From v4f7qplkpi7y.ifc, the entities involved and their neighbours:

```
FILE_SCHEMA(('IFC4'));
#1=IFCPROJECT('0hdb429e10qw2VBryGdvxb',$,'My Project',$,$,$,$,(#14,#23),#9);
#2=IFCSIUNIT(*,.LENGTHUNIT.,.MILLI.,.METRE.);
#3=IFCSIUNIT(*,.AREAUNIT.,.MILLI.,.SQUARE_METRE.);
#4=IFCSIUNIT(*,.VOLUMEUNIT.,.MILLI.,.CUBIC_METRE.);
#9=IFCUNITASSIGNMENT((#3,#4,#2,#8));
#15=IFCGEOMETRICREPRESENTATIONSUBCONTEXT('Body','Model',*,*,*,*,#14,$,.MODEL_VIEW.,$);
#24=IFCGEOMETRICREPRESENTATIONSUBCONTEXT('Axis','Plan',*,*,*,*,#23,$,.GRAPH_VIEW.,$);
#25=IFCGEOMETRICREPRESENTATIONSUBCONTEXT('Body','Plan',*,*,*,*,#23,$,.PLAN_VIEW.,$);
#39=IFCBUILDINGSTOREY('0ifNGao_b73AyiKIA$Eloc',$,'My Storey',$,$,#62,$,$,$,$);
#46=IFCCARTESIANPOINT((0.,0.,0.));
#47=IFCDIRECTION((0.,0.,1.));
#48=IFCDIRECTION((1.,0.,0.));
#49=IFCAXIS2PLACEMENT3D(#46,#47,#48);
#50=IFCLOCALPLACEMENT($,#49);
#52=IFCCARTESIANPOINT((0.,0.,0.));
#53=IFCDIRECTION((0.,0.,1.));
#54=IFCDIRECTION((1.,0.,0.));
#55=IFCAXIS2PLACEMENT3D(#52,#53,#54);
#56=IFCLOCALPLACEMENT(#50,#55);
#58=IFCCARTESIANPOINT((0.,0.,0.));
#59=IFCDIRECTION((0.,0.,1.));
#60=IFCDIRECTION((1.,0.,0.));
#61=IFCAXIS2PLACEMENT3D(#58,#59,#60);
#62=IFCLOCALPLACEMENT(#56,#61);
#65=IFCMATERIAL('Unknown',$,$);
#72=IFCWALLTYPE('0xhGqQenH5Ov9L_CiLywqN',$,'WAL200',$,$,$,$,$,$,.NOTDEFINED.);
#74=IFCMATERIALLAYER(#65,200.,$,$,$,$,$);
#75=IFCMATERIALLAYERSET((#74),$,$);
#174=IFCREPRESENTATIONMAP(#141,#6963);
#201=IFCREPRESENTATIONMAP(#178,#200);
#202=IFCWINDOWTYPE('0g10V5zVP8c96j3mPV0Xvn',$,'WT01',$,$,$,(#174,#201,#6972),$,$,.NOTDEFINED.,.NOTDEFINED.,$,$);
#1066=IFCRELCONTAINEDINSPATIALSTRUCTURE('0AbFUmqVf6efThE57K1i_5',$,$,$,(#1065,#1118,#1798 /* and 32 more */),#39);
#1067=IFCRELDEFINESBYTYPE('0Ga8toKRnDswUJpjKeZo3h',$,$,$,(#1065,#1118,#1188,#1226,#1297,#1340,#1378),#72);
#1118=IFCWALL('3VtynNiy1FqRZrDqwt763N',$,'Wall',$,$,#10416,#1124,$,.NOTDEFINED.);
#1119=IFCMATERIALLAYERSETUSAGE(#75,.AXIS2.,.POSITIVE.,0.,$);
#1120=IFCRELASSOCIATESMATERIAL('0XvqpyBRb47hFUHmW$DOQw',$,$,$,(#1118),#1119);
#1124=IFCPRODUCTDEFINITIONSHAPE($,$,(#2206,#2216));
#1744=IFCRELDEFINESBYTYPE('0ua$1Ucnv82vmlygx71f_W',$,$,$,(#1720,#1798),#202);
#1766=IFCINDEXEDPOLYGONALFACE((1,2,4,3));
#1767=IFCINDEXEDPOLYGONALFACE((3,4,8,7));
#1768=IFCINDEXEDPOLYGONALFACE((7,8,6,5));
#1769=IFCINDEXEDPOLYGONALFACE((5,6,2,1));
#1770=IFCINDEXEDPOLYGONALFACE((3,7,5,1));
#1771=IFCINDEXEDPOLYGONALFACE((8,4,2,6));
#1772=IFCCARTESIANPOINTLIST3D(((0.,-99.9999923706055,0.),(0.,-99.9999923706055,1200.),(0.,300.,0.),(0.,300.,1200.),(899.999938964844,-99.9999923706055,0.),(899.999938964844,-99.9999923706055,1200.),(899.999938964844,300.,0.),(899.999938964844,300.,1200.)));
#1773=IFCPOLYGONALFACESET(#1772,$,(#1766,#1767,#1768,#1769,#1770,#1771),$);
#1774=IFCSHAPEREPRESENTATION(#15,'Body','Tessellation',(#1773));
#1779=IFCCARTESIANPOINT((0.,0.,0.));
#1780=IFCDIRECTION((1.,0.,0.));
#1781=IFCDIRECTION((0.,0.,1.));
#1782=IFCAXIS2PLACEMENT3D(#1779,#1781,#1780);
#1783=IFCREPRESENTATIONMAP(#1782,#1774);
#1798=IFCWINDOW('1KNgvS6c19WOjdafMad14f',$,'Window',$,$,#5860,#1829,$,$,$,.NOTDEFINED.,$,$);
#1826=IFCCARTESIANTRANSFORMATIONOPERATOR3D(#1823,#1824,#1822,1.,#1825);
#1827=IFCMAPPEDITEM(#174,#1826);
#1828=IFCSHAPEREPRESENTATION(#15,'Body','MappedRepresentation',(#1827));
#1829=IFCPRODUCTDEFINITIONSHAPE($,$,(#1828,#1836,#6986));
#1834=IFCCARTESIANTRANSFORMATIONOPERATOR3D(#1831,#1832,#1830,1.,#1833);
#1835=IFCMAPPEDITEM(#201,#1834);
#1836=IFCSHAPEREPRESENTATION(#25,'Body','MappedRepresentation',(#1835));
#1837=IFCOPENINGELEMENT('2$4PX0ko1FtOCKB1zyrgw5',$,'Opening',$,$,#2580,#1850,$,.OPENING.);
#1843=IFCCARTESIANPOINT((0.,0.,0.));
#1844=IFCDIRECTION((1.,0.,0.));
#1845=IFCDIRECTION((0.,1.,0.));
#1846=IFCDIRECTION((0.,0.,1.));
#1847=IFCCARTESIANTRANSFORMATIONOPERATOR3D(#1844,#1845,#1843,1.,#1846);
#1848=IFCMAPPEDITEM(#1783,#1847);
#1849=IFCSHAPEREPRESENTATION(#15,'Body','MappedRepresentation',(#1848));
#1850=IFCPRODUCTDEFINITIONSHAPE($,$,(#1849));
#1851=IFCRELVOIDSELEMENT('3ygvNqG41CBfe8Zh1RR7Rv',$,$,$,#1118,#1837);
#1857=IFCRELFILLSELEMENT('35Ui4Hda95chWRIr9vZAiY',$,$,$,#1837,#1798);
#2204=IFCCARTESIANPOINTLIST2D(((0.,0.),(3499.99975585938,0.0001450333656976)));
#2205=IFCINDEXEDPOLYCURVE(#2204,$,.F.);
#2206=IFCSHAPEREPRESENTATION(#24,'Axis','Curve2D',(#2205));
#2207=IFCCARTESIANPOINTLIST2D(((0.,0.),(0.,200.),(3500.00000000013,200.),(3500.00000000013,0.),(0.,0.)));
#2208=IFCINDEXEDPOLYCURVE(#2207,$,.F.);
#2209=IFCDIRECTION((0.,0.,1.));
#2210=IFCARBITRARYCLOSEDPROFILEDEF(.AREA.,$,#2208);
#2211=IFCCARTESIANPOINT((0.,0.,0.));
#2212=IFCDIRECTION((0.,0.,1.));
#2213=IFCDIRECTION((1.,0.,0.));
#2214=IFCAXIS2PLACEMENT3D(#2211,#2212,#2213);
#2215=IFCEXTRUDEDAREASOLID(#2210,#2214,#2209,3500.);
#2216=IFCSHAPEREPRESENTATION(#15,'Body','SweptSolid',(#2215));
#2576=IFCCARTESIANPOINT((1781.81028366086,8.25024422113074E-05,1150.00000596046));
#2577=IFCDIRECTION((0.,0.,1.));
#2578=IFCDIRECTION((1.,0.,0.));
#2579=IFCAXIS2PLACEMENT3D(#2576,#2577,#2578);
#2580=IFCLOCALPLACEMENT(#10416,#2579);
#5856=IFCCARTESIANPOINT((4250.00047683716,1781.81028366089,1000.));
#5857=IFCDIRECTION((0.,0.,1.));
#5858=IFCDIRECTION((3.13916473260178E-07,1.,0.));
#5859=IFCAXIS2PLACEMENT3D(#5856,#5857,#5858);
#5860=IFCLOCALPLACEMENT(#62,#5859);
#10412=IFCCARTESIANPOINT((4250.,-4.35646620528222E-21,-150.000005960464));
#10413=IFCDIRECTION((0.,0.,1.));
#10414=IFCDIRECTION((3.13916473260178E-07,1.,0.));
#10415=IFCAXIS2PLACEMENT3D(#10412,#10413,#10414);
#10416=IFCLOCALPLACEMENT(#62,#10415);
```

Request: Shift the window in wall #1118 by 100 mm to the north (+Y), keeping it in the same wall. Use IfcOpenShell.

```python
import ifcopenshell
import ifcopenshell.api.geometry
import ifcopenshell.util.placement

model = ifcopenshell.open("v4f7qplkpi7y.ifc")

window = model.by_guid("1KNgvS6c19WOjdafMad14f")
opening = window.FillsVoids[0].RelatingOpeningElement
wall = opening.VoidsElements[0].RelatingBuildingElement

wall_matrix = ifcopenshell.util.placement.get_local_placement(wall.ObjectPlacement)
shift = wall_matrix[:3, 0] * 100.0
before = ifcopenshell.util.placement.get_local_placement(window.ObjectPlacement)[:3, 3].copy()

# The window is not placed relative to its opening, so move both.
for product in (opening, window):
    matrix = ifcopenshell.util.placement.get_local_placement(product.ObjectPlacement)
    matrix[:3, 3] += shift
    ifcopenshell.api.geometry.edit_object_placement(model, product=product, matrix=matrix, is_si=False)

after = ifcopenshell.util.placement.get_local_placement(window.ObjectPlacement)[:3, 3]
print("window moved by", (after - before).round(3) + 0.0)

model.write("v4f7qplkpi7y_updated.ifc")
```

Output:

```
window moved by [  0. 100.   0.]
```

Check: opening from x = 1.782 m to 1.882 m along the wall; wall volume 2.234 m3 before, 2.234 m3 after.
